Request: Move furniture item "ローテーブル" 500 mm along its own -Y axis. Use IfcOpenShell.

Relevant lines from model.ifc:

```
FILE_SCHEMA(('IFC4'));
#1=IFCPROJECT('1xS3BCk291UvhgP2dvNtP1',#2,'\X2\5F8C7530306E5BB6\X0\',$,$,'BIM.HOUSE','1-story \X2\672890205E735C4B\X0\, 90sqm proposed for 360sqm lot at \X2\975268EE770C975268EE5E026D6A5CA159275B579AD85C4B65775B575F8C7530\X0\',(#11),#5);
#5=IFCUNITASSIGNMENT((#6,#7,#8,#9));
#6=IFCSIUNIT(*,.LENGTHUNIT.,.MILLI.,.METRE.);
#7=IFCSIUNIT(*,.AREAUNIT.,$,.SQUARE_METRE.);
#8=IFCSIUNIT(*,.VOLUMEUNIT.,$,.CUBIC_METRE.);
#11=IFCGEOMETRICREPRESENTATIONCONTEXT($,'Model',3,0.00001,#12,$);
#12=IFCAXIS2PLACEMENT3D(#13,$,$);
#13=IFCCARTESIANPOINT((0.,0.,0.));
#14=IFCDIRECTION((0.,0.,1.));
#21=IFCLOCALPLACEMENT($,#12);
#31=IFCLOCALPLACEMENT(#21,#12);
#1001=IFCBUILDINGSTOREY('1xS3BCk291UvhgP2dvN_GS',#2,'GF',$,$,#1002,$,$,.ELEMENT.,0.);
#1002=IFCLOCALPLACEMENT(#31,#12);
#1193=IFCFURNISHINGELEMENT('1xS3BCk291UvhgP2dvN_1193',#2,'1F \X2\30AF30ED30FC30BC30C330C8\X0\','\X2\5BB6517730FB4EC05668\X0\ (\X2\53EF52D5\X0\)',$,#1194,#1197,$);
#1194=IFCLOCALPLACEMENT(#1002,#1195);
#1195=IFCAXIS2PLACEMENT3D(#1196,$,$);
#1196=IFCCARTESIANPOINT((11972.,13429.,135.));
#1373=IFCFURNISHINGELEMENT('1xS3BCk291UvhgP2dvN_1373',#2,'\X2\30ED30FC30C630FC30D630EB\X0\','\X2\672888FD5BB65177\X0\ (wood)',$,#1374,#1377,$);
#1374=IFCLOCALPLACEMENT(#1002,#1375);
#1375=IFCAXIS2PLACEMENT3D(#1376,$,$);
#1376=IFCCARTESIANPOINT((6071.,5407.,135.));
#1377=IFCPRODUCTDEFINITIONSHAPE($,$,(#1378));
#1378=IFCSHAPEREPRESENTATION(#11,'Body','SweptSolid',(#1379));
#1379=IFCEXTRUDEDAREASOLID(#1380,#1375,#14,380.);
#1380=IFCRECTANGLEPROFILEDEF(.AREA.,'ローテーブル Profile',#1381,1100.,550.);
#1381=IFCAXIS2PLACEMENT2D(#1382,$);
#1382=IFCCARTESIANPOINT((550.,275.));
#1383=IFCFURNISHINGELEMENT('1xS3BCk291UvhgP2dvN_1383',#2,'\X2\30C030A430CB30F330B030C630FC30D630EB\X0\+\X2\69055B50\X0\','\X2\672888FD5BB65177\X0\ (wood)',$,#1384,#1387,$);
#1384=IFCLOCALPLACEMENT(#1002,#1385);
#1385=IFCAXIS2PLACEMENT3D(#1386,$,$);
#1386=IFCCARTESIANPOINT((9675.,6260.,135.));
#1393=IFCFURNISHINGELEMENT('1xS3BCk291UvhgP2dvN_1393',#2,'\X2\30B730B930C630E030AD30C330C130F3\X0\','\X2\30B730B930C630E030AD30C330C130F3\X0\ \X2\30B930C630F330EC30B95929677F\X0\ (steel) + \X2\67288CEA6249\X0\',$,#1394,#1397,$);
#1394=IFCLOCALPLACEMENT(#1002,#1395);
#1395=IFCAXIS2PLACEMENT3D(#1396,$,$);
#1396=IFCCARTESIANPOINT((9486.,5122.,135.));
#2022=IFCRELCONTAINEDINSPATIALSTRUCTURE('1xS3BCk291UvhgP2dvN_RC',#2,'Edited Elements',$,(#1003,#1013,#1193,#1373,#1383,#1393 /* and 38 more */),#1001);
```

```python
import ifcopenshell
import ifcopenshell.api.geometry
import ifcopenshell.util.placement

model = ifcopenshell.open("model.ifc")

item = model.by_id(1373)
matrix = ifcopenshell.util.placement.get_local_placement(item.ObjectPlacement)
matrix[:3, 3] -= matrix[:3, 1] * 500.0
ifcopenshell.api.geometry.edit_object_placement(model, product=item, matrix=matrix, is_si=False)

print(ifcopenshell.util.placement.get_local_placement(item.ObjectPlacement).round(3) + 0.0)

model.write("model_rev.ifc")
```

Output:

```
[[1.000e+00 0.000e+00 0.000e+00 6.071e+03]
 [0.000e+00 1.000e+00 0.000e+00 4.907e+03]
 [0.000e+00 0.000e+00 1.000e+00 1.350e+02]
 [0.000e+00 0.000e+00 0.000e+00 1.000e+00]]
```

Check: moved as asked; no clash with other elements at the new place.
